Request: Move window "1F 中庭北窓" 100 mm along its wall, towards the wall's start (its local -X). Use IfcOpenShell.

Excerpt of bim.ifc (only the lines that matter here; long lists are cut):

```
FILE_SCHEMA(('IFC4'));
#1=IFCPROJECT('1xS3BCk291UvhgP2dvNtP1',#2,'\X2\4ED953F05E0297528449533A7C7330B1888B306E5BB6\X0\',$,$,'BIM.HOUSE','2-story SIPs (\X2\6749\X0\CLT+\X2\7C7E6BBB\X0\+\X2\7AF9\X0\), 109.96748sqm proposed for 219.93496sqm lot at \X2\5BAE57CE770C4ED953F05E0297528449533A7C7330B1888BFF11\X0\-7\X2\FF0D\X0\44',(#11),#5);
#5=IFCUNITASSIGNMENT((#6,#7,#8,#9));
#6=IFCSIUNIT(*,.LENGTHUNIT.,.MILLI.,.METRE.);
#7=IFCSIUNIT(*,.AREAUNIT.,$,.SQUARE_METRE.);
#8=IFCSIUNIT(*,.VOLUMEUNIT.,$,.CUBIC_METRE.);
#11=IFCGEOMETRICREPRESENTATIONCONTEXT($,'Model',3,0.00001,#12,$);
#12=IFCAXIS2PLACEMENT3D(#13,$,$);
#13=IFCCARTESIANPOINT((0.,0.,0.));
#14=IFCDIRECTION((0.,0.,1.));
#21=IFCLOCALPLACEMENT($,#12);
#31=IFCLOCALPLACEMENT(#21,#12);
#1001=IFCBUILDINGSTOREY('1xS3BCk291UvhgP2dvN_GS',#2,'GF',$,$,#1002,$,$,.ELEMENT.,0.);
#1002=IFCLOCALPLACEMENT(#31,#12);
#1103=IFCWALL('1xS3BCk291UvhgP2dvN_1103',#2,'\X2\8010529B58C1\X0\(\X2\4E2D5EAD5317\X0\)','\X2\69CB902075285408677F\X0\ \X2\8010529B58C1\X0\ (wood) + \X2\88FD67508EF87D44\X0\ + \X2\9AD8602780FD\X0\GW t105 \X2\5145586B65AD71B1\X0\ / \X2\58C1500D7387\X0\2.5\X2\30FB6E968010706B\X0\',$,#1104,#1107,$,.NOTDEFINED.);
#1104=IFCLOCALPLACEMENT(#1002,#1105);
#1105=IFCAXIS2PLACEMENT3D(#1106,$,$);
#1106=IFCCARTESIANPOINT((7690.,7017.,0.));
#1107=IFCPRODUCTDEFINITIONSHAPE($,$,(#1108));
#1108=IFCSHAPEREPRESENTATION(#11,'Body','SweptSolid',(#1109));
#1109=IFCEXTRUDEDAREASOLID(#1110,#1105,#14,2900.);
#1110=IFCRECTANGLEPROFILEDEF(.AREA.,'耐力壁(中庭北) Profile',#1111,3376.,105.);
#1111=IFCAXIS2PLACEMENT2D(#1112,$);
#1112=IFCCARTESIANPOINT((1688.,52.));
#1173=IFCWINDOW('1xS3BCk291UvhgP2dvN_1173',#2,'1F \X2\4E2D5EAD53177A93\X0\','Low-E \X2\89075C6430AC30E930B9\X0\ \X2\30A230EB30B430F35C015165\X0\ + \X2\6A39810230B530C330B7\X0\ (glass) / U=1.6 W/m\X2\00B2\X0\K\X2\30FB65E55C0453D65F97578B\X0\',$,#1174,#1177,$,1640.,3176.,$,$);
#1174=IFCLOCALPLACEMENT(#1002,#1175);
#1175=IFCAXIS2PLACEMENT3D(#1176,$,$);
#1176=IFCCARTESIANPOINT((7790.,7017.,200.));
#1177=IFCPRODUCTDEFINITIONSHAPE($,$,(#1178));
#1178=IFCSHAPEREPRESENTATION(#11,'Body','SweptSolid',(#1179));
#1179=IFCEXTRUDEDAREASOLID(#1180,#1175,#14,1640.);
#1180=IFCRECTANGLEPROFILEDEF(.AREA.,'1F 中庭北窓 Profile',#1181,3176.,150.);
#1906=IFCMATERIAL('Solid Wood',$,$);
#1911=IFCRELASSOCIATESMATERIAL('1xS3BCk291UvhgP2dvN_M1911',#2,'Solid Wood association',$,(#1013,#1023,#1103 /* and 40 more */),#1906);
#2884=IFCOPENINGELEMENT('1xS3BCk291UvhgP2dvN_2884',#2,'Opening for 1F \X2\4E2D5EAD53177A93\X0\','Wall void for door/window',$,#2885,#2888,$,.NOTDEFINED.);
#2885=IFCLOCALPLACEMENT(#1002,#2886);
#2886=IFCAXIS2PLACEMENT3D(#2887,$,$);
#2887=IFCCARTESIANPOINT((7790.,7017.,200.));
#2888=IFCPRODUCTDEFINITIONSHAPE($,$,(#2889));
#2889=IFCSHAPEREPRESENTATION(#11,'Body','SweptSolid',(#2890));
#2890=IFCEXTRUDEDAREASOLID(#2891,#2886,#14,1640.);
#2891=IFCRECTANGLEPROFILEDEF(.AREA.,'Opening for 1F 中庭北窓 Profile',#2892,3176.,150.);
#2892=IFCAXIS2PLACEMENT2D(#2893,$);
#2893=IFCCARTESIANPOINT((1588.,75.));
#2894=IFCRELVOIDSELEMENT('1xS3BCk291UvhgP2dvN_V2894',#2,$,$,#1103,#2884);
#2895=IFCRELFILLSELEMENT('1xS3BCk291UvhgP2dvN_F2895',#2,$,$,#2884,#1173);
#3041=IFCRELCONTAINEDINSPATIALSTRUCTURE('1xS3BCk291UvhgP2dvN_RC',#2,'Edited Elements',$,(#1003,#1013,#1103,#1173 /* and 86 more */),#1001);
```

```python
import ifcopenshell
import ifcopenshell.api.geometry
import ifcopenshell.util.placement
import ifcopenshell.util.unit

model = ifcopenshell.open("bim.ifc")
unit_scale = ifcopenshell.util.unit.calculate_unit_scale(model)

window = model.by_guid("1xS3BCk291UvhgP2dvN_1173")
opening = window.FillsVoids[0].RelatingOpeningElement
wall = opening.VoidsElements[0].RelatingBuildingElement

wall_matrix = ifcopenshell.util.placement.get_local_placement(wall.ObjectPlacement)
shift = wall_matrix[:3, 0] * -0.1 / unit_scale
before = ifcopenshell.util.placement.get_local_placement(window.ObjectPlacement)[:3, 3].copy()

# The window is not placed relative to its opening, so move both.
for product in (opening, window):
    matrix = ifcopenshell.util.placement.get_local_placement(product.ObjectPlacement)
    matrix[:3, 3] += shift
    ifcopenshell.api.geometry.edit_object_placement(model, product=product, matrix=matrix, is_si=False)

after = ifcopenshell.util.placement.get_local_placement(window.ObjectPlacement)[:3, 3]
print("window moved by", (after - before).round(3) + 0.0)

model.write("bim_v2.ifc")
```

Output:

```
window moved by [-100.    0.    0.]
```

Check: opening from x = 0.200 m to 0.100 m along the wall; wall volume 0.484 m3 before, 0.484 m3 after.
